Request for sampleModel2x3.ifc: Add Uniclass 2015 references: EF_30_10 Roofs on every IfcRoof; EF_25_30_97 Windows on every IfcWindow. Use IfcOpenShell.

First a look at what the model holds.

```python
import ifcopenshell

model = ifcopenshell.open("sampleModel2x3.ifc")
print(model.schema)
print("classifications:", [c.Name for c in model.by_type("IfcClassification")])
for ifc_class in ("IfcDoor", "IfcRoof", "IfcStair", "IfcWall", "IfcWindow"):
    print(ifc_class, len(model.by_type(ifc_class)))
```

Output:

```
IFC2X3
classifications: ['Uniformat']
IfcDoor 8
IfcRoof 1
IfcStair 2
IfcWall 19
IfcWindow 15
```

```python
import ifcopenshell
import ifcopenshell.api.classification

model = ifcopenshell.open("sampleModel2x3.ifc")

# IFC2X3 requires Source and Edition and has no link from the project to the system.
system = model.create_entity("IfcClassification", Source="NBS", Edition="2015", Name="Uniclass 2015")

codes = {
    "IfcRoof": ("EF_30_10", "Roofs"),
    "IfcWindow": ("EF_25_30_97", "Windows"),
}
for ifc_class, (code, name) in codes.items():
    products = model.by_type(ifc_class)
    ifcopenshell.api.classification.add_reference(
        model, products=products, classification=system, identification=code, name=name
    )
    print(code, len(products))

model.write("sampleModel2x3_edited.ifc")
```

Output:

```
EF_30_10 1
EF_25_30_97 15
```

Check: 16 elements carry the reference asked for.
